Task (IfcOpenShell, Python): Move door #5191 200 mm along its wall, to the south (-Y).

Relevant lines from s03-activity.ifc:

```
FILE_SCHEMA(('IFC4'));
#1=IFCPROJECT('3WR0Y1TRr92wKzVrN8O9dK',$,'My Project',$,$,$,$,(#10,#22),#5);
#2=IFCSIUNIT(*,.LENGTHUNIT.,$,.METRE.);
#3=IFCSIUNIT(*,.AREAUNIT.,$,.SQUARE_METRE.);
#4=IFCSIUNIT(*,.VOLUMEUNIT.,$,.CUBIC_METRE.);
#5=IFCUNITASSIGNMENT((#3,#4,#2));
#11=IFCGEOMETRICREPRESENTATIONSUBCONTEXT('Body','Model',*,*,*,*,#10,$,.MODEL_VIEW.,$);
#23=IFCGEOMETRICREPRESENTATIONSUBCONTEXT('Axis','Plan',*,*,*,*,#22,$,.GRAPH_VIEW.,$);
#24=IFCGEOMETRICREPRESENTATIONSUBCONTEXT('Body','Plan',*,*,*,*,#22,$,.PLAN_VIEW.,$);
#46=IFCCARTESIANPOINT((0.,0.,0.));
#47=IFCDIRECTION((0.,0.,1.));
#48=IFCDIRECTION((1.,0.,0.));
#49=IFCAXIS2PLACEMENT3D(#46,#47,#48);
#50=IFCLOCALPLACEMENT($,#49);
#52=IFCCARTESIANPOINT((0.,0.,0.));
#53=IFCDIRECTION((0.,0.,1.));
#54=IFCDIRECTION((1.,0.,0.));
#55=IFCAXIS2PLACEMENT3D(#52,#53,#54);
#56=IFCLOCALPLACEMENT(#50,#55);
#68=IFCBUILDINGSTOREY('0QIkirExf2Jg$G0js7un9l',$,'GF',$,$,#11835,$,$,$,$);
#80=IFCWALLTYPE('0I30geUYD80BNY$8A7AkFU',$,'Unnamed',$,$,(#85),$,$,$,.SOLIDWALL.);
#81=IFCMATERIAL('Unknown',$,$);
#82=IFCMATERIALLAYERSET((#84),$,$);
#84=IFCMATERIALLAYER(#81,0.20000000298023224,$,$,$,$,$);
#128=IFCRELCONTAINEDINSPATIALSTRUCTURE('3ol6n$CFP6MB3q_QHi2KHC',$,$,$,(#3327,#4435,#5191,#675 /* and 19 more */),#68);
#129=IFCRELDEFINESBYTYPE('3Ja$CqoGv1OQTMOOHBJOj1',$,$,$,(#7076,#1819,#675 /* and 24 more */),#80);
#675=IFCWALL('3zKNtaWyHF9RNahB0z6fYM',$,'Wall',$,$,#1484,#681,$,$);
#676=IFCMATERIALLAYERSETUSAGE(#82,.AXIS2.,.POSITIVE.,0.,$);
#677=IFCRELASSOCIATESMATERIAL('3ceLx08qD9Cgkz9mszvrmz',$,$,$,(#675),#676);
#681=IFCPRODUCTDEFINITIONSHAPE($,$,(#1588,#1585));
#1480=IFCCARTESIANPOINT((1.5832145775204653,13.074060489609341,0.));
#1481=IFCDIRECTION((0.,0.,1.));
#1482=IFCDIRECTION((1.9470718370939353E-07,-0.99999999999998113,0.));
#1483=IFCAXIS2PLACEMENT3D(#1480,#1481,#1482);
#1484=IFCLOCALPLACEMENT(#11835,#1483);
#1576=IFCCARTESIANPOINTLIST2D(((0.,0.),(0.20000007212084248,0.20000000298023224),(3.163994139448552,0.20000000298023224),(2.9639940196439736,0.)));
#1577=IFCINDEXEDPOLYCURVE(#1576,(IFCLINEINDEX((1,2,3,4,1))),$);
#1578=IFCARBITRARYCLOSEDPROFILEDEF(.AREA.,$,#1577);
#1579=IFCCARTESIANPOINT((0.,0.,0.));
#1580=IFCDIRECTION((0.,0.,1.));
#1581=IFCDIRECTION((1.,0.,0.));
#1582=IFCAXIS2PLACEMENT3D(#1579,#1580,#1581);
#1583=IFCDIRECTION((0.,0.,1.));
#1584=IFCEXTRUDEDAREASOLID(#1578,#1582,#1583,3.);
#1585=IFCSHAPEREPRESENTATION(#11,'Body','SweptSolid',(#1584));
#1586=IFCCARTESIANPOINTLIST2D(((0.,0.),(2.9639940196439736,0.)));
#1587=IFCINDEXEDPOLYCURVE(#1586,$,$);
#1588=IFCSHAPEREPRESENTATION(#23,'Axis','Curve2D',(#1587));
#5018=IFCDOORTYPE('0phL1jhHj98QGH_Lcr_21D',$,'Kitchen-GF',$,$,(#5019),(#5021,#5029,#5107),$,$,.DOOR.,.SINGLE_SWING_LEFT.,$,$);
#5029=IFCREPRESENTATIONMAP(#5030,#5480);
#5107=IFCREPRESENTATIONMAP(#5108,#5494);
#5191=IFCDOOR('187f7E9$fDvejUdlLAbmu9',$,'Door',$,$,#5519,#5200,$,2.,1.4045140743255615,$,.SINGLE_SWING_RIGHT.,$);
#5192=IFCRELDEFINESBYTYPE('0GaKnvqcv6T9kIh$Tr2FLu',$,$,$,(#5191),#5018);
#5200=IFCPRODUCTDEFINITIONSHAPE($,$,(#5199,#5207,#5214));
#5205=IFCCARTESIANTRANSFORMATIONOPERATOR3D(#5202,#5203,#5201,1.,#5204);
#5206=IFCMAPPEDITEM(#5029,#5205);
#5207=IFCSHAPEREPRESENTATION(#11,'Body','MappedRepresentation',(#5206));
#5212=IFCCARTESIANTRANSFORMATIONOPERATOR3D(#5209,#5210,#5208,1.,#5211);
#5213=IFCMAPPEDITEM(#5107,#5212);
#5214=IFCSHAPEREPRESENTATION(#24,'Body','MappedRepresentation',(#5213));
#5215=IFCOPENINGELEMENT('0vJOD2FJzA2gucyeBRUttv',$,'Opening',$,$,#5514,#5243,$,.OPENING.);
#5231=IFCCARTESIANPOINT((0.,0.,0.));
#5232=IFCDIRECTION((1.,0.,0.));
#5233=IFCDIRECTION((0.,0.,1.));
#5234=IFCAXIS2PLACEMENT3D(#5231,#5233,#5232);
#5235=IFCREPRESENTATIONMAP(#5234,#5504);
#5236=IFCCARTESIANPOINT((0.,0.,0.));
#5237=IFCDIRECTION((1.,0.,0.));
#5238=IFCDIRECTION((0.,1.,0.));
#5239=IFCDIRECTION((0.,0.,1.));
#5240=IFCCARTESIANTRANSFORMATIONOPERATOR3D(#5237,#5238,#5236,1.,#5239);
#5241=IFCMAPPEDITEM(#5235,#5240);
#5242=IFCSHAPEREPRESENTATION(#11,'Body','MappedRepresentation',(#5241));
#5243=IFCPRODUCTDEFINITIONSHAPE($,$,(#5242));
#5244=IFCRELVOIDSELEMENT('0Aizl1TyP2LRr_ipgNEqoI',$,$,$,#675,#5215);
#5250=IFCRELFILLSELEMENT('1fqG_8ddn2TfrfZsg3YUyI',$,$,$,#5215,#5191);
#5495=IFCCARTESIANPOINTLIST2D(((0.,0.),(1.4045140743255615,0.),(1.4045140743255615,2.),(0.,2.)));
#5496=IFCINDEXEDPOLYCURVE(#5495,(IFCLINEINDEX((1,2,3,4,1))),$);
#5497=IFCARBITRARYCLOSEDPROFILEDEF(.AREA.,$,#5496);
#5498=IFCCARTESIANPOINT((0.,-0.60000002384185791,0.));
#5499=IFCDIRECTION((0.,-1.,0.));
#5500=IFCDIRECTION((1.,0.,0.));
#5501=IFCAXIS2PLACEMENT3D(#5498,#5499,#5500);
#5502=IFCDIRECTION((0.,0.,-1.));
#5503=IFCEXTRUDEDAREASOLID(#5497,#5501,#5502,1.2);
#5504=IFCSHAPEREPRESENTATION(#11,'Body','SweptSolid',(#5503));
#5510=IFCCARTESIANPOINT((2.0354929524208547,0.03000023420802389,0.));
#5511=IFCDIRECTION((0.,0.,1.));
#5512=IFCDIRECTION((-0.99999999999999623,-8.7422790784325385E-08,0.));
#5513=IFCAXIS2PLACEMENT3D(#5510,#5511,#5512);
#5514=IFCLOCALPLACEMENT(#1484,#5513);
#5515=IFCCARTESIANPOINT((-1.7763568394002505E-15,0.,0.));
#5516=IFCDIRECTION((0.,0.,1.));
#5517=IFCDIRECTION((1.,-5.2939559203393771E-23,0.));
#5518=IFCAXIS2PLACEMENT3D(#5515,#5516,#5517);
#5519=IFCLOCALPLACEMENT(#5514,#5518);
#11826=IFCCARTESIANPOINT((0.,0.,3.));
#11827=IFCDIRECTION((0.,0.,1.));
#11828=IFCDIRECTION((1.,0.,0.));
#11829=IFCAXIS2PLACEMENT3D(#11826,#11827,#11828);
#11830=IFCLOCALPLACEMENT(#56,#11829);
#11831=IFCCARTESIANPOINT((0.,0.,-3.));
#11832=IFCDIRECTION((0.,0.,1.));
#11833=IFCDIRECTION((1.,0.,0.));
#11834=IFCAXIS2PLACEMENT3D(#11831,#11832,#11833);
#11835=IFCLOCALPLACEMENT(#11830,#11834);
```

```python
import ifcopenshell
import ifcopenshell.api.geometry
import ifcopenshell.util.placement

model = ifcopenshell.open("s03-activity.ifc")

door = model.by_id(5191)
opening = door.FillsVoids[0].RelatingOpeningElement
wall = opening.VoidsElements[0].RelatingBuildingElement

wall_matrix = ifcopenshell.util.placement.get_local_placement(wall.ObjectPlacement)
shift = wall_matrix[:3, 0] * 0.2
before = ifcopenshell.util.placement.get_local_placement(door.ObjectPlacement)[:3, 3].copy()

# The door is placed relative to its opening, so it follows when the opening moves.
matrix = ifcopenshell.util.placement.get_local_placement(opening.ObjectPlacement)
matrix[:3, 3] += shift
ifcopenshell.api.geometry.edit_object_placement(
    model, product=opening, matrix=matrix, is_si=False, should_transform_children=True
)

after = ifcopenshell.util.placement.get_local_placement(door.ObjectPlacement)[:3, 3]
print("door moved by", (after - before).round(3) + 0.0)

model.write("s03-activity_rev.ifc")
```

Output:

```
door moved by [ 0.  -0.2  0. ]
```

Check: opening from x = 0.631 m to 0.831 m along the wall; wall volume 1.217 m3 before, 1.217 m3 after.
